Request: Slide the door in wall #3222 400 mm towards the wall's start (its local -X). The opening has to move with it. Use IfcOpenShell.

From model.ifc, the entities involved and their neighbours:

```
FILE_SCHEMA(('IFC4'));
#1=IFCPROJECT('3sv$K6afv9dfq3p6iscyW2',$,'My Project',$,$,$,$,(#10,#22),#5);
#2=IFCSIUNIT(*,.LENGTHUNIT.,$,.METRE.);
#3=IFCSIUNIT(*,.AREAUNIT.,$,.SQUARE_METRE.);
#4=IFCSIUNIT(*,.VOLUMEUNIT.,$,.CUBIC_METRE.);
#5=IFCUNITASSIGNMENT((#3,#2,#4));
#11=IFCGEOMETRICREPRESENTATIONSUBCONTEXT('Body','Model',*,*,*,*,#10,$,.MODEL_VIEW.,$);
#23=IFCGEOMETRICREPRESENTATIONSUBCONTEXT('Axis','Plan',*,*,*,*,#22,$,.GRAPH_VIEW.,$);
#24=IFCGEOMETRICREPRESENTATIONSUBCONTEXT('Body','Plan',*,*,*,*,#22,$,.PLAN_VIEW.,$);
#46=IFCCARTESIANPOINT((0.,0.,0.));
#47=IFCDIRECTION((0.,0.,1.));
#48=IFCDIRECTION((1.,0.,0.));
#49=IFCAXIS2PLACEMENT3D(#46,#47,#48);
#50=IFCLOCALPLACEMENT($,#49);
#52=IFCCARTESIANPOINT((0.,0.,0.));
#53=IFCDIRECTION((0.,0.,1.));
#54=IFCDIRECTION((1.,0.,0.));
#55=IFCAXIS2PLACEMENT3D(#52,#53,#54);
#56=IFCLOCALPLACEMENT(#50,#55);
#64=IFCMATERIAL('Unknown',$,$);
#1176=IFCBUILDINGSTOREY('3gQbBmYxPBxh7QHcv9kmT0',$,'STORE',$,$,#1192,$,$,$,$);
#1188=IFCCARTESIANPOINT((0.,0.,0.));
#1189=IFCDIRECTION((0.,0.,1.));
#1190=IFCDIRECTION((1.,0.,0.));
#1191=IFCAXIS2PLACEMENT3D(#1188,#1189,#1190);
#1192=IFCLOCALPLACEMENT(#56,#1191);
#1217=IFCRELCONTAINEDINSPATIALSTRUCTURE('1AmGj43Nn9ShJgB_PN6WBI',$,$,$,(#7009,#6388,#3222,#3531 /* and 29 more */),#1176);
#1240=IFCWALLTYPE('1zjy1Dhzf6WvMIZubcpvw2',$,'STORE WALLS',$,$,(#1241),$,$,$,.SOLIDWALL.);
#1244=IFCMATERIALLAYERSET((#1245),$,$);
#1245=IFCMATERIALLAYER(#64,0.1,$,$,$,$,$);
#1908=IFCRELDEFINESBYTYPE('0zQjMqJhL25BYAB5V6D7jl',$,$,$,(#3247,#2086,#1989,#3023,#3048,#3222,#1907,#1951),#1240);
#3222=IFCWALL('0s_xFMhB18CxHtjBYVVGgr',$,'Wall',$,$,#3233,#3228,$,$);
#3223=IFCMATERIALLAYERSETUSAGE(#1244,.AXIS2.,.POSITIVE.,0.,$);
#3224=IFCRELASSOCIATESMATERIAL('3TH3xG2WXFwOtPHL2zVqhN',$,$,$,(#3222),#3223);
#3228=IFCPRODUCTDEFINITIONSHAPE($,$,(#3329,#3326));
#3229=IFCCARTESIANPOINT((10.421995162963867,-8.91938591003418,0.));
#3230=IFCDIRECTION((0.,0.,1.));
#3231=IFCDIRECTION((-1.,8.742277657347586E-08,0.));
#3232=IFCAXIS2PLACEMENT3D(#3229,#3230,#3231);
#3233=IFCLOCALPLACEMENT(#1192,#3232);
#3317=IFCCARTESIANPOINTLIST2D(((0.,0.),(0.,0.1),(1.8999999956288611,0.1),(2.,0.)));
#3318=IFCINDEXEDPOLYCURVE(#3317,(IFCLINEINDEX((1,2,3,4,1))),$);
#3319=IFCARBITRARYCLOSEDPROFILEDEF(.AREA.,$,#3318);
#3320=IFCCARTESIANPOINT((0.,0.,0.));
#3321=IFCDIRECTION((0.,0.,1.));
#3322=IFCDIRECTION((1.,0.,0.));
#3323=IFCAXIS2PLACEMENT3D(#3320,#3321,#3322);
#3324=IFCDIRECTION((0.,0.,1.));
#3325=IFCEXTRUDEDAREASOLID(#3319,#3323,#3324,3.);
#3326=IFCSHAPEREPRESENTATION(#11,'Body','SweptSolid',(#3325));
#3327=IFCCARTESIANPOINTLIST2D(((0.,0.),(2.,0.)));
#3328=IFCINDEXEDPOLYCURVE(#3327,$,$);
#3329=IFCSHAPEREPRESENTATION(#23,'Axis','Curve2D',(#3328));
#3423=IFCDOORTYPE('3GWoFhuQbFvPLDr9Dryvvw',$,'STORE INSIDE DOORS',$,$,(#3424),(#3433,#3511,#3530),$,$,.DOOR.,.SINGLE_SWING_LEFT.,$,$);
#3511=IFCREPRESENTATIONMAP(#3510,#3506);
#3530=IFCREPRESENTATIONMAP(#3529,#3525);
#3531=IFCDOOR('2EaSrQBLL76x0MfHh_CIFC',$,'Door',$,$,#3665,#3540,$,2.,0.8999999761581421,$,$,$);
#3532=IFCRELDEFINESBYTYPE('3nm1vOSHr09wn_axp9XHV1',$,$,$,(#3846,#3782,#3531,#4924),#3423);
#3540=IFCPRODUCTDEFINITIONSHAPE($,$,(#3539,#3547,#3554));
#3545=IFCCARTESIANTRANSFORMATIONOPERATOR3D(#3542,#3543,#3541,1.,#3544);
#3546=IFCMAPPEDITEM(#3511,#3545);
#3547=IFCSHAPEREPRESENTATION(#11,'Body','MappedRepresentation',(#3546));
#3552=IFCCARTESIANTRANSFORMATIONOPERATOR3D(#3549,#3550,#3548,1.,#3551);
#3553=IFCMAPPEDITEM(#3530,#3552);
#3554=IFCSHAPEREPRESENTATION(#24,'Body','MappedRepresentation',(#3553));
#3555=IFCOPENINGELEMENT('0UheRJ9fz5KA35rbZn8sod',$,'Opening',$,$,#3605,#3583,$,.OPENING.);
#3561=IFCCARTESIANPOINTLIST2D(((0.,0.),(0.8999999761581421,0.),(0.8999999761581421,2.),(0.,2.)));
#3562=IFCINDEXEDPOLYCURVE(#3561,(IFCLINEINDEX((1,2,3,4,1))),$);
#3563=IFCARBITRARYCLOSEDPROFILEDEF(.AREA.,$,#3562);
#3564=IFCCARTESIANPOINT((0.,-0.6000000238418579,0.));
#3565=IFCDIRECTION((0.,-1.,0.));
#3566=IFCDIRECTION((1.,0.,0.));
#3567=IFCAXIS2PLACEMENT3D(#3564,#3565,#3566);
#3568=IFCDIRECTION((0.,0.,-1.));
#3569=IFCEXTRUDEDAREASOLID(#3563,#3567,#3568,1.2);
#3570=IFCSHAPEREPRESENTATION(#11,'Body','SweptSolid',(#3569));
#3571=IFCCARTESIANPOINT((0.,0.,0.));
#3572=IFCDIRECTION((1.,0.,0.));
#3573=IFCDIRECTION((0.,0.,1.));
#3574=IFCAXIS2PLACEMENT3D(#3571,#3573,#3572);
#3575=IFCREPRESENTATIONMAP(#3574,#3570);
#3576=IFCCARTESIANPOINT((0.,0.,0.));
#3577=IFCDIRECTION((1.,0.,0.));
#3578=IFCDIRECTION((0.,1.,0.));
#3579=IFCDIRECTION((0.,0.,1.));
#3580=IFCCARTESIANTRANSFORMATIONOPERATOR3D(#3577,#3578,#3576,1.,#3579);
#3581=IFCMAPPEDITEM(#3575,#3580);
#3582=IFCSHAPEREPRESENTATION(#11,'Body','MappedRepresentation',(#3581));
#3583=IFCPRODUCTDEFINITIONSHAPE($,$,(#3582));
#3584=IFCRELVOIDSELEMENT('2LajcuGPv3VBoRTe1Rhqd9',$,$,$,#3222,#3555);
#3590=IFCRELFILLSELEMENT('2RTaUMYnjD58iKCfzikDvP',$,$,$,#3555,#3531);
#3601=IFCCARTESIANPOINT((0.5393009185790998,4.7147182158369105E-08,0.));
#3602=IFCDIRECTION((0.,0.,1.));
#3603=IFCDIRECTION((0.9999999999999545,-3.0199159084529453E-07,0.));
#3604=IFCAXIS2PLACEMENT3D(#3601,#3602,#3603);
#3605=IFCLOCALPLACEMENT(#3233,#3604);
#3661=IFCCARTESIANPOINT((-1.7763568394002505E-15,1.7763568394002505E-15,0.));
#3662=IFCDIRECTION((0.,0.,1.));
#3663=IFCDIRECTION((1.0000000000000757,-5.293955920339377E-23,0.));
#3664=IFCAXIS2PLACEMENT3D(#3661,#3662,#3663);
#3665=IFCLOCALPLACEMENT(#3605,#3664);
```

```python
import ifcopenshell
import ifcopenshell.api.geometry
import ifcopenshell.util.placement

model = ifcopenshell.open("model.ifc")

door = model.by_id(3531)
opening = door.FillsVoids[0].RelatingOpeningElement
wall = opening.VoidsElements[0].RelatingBuildingElement

wall_matrix = ifcopenshell.util.placement.get_local_placement(wall.ObjectPlacement)
shift = wall_matrix[:3, 0] * -0.4
before = ifcopenshell.util.placement.get_local_placement(door.ObjectPlacement)[:3, 3].copy()

# The door is placed relative to its opening, so it follows when the opening moves.
matrix = ifcopenshell.util.placement.get_local_placement(opening.ObjectPlacement)
matrix[:3, 3] += shift
ifcopenshell.api.geometry.edit_object_placement(
    model, product=opening, matrix=matrix, is_si=False, should_transform_children=True
)

after = ifcopenshell.util.placement.get_local_placement(door.ObjectPlacement)[:3, 3]
print("door moved by", (after - before).round(3) + 0.0)

model.write("model_updated.ifc")
```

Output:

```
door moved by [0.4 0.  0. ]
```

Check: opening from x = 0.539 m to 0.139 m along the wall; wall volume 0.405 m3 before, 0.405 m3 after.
